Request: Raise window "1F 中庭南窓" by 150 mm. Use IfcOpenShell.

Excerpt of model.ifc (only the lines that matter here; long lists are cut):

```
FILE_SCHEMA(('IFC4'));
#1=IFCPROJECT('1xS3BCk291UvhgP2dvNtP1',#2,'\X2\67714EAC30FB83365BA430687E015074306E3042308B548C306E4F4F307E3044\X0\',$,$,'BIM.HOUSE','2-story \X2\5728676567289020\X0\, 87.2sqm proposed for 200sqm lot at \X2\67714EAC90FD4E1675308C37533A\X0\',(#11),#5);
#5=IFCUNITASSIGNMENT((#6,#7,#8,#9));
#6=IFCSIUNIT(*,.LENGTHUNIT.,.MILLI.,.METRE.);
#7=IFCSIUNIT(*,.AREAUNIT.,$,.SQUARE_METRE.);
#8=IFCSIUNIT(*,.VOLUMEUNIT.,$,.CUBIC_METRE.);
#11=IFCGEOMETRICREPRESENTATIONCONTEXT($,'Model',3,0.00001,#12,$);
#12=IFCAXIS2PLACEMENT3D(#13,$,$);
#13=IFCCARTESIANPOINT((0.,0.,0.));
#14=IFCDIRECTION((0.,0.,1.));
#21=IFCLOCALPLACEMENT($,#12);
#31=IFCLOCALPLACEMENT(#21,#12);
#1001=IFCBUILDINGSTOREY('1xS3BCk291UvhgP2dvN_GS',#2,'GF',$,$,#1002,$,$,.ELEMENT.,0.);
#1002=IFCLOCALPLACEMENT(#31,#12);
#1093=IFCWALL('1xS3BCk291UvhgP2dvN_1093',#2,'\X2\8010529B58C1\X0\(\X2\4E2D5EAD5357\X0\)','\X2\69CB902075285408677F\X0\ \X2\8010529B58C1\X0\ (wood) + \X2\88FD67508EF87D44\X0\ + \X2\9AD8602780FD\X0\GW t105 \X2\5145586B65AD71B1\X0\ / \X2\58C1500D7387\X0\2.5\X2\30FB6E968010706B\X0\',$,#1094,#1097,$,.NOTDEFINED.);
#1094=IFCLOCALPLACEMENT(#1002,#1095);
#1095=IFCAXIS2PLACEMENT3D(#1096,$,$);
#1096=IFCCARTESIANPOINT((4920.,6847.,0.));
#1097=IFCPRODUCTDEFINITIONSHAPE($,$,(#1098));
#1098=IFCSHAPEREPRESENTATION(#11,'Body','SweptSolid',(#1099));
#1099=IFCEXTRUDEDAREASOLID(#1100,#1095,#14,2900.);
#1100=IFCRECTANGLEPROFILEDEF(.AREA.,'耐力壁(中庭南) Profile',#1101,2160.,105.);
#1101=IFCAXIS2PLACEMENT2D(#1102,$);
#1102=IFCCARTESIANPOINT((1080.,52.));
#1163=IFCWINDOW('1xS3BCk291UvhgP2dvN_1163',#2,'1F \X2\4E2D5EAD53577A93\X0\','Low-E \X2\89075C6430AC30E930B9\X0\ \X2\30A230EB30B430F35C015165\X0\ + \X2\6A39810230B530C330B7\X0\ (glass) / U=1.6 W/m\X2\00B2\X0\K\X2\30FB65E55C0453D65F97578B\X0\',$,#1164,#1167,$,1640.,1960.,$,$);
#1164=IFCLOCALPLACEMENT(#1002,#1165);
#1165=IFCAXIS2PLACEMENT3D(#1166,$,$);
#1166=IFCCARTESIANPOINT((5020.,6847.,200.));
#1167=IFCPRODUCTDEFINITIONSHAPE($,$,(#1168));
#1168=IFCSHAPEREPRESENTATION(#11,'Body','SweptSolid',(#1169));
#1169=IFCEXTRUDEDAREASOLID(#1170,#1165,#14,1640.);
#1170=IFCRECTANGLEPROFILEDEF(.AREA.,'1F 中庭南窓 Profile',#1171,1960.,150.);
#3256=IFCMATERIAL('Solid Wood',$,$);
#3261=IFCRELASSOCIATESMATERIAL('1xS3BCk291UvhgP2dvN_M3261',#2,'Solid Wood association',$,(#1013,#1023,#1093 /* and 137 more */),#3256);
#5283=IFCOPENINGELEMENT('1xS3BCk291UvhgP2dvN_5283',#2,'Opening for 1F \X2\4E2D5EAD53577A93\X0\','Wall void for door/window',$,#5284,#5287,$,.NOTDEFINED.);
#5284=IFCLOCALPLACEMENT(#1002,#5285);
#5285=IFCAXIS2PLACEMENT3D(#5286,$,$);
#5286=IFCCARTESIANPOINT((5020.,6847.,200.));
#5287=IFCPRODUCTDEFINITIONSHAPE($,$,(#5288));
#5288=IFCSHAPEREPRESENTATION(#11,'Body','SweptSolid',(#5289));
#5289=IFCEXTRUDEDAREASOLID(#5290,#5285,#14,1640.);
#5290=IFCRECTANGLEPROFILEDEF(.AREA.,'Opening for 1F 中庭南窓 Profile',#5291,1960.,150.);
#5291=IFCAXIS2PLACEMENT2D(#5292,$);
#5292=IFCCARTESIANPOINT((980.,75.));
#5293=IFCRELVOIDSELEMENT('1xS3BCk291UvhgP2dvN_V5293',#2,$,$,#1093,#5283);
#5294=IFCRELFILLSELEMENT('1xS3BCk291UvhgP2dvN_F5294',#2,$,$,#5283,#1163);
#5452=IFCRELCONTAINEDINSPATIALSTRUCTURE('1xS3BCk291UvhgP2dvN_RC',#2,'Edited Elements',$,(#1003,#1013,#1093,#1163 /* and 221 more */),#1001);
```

```python
import numpy as np
import ifcopenshell
import ifcopenshell.api.geometry
import ifcopenshell.util.placement
import ifcopenshell.util.unit

model = ifcopenshell.open("model.ifc")
unit_scale = ifcopenshell.util.unit.calculate_unit_scale(model)

window = model.by_guid("1xS3BCk291UvhgP2dvN_1163")
opening = window.FillsVoids[0].RelatingOpeningElement
dz = 150.0

shift = np.array([0.0, 0.0, dz])
# The window is not placed relative to its opening, so move both.
for product in (opening, window):
    matrix = ifcopenshell.util.placement.get_local_placement(product.ObjectPlacement)
    matrix[:3, 3] += shift
    ifcopenshell.api.geometry.edit_object_placement(model, product=product, matrix=matrix, is_si=False)

print(f"moved by {dz * unit_scale:+.3f} m")

model.write("model_v2.ifc")
```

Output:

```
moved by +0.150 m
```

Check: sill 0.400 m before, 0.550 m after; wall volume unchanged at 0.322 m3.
